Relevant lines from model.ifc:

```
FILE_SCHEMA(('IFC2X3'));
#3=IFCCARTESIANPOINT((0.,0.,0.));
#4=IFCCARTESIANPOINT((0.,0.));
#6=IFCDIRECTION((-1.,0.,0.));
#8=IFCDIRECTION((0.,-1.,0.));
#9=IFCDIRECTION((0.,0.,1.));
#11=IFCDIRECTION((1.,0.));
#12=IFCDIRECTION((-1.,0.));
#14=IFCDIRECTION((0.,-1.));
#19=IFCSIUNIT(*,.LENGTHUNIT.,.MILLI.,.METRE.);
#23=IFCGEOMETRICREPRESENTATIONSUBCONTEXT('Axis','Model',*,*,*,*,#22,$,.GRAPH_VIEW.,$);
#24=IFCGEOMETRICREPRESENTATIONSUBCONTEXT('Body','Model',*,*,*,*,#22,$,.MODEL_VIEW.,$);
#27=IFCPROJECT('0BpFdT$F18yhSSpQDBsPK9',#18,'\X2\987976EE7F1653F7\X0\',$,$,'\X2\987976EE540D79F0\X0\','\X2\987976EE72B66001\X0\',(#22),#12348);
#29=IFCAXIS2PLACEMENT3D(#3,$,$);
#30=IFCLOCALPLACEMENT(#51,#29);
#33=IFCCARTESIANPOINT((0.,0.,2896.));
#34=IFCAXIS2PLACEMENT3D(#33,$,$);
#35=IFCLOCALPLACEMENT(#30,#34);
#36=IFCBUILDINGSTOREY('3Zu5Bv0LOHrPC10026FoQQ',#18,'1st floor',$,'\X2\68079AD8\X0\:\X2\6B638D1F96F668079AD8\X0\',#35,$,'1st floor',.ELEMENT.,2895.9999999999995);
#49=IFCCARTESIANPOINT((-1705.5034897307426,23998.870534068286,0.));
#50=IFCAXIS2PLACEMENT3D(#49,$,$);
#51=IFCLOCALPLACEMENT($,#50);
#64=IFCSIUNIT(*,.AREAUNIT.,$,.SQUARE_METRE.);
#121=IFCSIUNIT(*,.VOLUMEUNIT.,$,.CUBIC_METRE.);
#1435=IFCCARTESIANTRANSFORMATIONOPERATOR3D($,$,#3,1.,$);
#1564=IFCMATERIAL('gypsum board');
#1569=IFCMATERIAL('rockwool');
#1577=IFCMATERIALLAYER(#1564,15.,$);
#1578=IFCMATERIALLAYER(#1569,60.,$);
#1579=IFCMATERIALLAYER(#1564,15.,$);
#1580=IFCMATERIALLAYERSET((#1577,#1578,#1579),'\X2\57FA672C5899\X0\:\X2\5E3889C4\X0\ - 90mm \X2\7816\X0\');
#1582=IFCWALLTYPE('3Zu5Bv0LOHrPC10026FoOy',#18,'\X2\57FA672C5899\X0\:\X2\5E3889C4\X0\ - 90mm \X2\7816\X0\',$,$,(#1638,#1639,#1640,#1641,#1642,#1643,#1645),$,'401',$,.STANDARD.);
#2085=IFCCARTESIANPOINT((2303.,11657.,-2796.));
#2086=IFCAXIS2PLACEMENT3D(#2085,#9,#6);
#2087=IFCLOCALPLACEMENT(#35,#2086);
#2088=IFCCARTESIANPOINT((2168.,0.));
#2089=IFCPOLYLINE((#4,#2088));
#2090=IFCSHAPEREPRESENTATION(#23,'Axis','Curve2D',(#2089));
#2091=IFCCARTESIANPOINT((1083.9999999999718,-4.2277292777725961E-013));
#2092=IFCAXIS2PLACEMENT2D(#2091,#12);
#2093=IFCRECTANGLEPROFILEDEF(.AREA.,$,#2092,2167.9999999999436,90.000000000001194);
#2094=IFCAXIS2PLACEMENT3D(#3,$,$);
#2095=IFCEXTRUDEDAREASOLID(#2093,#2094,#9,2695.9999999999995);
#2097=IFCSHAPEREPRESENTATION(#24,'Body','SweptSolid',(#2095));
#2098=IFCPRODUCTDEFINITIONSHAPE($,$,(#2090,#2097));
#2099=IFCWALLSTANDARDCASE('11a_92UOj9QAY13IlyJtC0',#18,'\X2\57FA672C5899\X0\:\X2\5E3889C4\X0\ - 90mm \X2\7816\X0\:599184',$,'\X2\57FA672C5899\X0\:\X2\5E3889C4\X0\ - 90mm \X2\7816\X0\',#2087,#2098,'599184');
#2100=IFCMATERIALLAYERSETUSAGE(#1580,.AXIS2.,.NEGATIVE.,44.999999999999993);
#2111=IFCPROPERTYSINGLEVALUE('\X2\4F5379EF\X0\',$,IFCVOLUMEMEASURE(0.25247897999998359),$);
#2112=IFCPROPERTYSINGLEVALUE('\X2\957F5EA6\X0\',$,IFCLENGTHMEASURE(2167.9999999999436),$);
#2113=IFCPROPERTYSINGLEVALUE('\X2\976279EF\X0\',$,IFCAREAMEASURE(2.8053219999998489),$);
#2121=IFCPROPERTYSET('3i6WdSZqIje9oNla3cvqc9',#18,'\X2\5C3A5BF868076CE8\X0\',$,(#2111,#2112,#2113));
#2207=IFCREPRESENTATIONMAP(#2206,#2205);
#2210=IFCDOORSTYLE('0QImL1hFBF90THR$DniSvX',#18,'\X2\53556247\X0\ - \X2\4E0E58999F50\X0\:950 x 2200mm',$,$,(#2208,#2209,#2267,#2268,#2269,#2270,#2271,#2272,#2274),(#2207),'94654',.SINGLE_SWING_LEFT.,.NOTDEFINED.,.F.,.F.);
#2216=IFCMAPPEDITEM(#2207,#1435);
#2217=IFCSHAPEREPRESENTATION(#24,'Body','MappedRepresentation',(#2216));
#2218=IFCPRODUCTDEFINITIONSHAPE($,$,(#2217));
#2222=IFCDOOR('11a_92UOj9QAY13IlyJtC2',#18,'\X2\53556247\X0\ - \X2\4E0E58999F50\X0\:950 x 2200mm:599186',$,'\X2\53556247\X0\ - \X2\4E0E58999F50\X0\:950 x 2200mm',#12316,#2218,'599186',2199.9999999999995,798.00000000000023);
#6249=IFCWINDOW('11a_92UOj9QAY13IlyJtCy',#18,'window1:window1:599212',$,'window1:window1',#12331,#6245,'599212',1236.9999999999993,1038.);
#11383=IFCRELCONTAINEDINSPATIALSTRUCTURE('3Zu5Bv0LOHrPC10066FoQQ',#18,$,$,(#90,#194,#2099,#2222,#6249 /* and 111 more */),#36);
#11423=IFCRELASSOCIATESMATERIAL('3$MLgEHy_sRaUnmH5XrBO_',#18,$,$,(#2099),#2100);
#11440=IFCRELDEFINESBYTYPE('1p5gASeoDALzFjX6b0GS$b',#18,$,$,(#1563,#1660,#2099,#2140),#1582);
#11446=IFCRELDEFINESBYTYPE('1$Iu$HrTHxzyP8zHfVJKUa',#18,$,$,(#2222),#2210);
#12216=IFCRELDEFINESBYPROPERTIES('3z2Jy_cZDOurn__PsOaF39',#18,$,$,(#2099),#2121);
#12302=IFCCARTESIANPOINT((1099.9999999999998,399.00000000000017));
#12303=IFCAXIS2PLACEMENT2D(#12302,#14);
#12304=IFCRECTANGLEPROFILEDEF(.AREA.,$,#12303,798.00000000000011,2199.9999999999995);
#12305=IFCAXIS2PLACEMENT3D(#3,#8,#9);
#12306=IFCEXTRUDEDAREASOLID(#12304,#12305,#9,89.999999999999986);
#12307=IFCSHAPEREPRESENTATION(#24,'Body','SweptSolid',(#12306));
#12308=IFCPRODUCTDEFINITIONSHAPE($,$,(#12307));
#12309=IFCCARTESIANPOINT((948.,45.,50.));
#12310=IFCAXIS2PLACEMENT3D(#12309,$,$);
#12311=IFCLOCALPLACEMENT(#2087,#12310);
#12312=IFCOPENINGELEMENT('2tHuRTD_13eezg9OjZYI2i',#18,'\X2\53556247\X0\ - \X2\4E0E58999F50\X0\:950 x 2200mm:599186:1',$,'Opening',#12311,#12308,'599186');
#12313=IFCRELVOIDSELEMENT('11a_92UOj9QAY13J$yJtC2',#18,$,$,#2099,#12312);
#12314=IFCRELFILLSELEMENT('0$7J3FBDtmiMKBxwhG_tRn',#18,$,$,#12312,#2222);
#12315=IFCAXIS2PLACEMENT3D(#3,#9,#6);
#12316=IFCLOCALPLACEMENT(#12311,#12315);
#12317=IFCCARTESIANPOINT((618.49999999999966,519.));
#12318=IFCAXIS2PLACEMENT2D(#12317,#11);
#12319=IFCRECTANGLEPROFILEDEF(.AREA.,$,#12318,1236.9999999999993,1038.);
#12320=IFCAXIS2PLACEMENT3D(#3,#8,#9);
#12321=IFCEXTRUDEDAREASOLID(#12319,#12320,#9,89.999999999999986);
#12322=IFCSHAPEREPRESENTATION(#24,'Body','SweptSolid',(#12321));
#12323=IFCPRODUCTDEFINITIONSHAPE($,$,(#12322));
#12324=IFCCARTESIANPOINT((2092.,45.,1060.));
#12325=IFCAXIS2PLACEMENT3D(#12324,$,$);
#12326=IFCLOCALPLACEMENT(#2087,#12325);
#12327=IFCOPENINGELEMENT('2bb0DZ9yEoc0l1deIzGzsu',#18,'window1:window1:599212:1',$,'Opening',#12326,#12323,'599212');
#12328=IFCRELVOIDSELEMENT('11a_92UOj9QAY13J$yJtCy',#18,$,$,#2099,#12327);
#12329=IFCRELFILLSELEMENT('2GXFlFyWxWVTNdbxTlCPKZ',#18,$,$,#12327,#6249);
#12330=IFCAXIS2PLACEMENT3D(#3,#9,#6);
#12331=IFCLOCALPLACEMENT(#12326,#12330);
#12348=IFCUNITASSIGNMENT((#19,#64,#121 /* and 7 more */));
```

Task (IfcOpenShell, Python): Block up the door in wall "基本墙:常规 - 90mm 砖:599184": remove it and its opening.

```python
import ifcopenshell
import ifcopenshell.api.feature
import ifcopenshell.api.pset
import ifcopenshell.api.root
import ifcopenshell.geom
import ifcopenshell.util.element
import ifcopenshell.util.shape
import ifcopenshell.util.unit

model = ifcopenshell.open("model.ifc")
area_scale = ifcopenshell.util.unit.calculate_unit_scale(model, "AREAUNIT")
volume_scale = ifcopenshell.util.unit.calculate_unit_scale(model, "VOLUMEUNIT")
settings = ifcopenshell.geom.settings()


def volume(element):
    """Net volume in cubic metres, openings subtracted."""
    shape = ifcopenshell.geom.create_shape(settings, element)
    return ifcopenshell.util.shape.get_volume(shape.geometry)


door = model.by_id(2222)
opening = door.FillsVoids[0].RelatingOpeningElement
wall = opening.VoidsElements[0].RelatingBuildingElement
before = volume(wall)

ifcopenshell.api.root.remove_product(model, product=door)
ifcopenshell.api.feature.remove_feature(model, feature=opening)

after = volume(wall)
thickness = 0.09  # wall thickness in metres

# Update the wall's stored quantities.
pset = model.by_id(ifcopenshell.util.element.get_pset(wall, "尺寸标注", should_inherit=False)["id"])
ifcopenshell.api.pset.edit_pset(model, pset=pset, properties={
    "体积": model.create_entity("IfcVolumeMeasure", after / volume_scale),
    "面积": model.create_entity("IfcAreaMeasure", after / thickness / area_scale),
})

print(f"wall volume {before:.3f} -> {after:.3f} m3")

model.write("model_updated.ifc")
```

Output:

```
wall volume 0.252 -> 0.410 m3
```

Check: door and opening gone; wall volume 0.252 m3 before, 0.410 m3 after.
